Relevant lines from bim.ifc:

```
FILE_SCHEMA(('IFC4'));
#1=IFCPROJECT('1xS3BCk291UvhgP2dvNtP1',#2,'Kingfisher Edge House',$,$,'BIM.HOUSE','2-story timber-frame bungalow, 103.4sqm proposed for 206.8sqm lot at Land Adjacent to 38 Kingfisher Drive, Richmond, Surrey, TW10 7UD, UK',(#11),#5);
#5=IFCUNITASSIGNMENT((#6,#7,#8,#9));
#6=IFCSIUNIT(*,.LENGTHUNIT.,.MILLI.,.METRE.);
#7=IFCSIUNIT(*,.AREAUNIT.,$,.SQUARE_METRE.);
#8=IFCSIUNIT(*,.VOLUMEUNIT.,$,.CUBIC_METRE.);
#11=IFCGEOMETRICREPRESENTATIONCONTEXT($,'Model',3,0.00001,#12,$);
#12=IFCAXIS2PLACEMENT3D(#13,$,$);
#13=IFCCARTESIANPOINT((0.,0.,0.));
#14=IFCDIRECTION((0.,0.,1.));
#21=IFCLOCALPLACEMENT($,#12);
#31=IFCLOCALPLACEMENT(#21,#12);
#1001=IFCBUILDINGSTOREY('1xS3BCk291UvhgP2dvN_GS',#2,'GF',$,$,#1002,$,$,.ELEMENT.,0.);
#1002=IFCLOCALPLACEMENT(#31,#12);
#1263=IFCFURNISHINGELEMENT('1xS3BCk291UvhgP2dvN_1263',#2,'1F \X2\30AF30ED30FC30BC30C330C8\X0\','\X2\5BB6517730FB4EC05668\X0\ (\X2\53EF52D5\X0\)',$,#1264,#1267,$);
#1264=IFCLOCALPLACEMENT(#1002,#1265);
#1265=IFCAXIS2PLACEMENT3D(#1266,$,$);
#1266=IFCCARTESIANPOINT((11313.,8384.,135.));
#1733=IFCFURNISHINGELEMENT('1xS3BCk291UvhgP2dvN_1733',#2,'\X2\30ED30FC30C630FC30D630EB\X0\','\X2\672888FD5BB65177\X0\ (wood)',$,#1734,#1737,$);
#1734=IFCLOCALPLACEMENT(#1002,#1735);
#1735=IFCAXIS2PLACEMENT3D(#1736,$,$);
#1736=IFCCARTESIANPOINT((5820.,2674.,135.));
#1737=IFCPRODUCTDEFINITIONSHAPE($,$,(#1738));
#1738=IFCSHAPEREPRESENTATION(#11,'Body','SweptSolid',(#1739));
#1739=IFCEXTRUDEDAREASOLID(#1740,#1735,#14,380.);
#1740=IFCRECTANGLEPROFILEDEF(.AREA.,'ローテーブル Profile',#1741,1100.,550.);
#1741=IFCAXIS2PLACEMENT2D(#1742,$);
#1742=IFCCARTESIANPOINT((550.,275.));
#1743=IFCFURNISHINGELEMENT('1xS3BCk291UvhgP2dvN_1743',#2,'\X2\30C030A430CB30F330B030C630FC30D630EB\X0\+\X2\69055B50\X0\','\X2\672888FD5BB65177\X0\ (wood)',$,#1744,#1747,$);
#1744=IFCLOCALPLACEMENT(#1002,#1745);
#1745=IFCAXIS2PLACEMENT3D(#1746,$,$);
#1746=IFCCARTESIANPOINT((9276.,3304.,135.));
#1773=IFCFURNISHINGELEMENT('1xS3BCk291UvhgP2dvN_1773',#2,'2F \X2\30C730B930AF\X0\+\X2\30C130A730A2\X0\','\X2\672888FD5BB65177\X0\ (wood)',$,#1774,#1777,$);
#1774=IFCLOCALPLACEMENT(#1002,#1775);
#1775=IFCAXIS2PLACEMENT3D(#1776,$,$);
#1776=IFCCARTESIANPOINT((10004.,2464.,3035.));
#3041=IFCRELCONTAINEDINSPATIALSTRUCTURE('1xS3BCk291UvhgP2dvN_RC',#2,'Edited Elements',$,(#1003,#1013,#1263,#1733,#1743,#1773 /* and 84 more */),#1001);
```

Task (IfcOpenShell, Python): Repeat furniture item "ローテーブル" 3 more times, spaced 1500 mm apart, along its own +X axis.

```python
import ifcopenshell
import ifcopenshell.api.geometry
import ifcopenshell.api.root
import ifcopenshell.util.element
import ifcopenshell.util.placement
import ifcopenshell.util.unit

model = ifcopenshell.open("bim.ifc")
unit_scale = ifcopenshell.util.unit.calculate_unit_scale(model)


def reuse_history(source, copy):
    """copy_class also copies each property set's owner history, people and application; keep the originals."""
    for rel in copy.IsDefinedBy:
        if rel.is_a("IfcRelDefinesByProperties") and (history := rel.RelatingPropertyDefinition.OwnerHistory):
            rel.RelatingPropertyDefinition.OwnerHistory = source.OwnerHistory
            ifcopenshell.util.element.remove_deep2(model, history)


source = model.by_guid("1xS3BCk291UvhgP2dvN_1733")
base = ifcopenshell.util.placement.get_local_placement(source.ObjectPlacement)
step = base[:3, 0] * 1.5 / unit_scale

for i in range(1, 4):
    copy = ifcopenshell.api.root.copy_class(model, product=source)
    copy.Representation = ifcopenshell.util.element.copy_deep(
        model, source.Representation, exclude=["IfcGeometricRepresentationContext", "IfcRepresentationMap"]
    )
    reuse_history(source, copy)
    matrix = base.copy()
    matrix[:3, 3] += i * step
    print("added at", matrix[:3, 3].round(3) + 0.0)
    ifcopenshell.api.geometry.edit_object_placement(model, product=copy, matrix=matrix, is_si=False)

model.write("bim_rev.ifc")
```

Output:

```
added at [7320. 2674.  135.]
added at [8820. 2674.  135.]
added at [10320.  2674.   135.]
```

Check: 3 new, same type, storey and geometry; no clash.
